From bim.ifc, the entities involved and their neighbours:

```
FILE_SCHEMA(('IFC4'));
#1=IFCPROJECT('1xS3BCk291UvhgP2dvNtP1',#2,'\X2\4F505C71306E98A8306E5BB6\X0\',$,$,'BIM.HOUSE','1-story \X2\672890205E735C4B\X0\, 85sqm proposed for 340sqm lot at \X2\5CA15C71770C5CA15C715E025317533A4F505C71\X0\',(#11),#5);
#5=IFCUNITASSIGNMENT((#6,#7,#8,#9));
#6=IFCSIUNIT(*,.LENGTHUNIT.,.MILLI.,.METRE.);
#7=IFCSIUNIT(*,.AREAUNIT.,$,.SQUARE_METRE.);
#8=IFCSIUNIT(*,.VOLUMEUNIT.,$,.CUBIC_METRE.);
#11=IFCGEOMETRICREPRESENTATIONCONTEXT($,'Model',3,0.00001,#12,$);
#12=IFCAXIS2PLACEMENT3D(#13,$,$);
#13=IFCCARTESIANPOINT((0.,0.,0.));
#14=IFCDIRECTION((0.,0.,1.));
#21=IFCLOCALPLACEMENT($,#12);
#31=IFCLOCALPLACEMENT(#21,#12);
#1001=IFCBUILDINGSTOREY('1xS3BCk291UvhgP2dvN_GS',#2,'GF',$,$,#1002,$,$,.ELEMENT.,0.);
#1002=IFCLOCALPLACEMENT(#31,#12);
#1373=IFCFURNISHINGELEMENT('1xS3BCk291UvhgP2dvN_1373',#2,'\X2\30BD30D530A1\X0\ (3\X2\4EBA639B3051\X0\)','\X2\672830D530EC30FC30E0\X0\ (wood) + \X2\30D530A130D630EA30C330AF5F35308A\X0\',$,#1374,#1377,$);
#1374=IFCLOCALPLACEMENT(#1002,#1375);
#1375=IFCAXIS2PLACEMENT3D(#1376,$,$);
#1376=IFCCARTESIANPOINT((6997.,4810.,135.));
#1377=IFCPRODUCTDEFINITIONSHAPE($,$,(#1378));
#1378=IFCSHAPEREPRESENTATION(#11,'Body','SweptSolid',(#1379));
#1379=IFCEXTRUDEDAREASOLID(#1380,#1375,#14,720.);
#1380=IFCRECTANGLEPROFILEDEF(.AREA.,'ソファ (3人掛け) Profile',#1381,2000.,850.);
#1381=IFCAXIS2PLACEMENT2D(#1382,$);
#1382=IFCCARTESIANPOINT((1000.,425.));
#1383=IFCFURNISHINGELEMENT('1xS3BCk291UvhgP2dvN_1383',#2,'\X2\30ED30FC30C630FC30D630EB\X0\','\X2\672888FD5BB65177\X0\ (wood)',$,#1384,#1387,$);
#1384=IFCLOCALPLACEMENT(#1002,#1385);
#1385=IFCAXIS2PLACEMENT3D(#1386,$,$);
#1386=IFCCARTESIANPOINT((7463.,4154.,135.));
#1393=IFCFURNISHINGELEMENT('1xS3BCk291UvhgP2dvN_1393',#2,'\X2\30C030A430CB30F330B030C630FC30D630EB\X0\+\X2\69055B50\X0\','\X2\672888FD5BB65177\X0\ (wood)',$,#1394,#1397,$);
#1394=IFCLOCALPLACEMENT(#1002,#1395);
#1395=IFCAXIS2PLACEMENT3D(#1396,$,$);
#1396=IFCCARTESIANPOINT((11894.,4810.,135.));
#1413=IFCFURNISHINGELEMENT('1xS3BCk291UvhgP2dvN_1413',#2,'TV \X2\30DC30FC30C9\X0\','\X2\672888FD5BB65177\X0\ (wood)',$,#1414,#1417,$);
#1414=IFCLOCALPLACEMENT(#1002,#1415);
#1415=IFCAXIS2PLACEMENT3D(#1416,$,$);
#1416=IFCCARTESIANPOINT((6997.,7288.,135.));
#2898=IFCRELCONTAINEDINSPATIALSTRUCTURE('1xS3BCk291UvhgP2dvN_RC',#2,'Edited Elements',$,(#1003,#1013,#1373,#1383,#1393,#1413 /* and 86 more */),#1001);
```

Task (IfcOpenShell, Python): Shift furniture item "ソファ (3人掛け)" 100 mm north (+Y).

```python
import ifcopenshell
import ifcopenshell.api.geometry
import ifcopenshell.util.placement

model = ifcopenshell.open("bim.ifc")

item = model.by_guid("1xS3BCk291UvhgP2dvN_1373")
matrix = ifcopenshell.util.placement.get_local_placement(item.ObjectPlacement)
matrix[1, 3] += 100.0
ifcopenshell.api.geometry.edit_object_placement(model, product=item, matrix=matrix, is_si=False)

print(ifcopenshell.util.placement.get_local_placement(item.ObjectPlacement).round(3) + 0.0)

model.write("bim-out.ifc")
```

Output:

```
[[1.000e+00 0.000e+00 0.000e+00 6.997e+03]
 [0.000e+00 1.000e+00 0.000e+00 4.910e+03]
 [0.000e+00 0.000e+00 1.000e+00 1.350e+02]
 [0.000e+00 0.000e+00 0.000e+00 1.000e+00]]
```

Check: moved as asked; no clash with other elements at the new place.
